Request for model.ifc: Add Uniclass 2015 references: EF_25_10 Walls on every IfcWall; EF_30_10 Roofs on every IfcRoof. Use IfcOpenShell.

First a look at what the model holds.

```python
import ifcopenshell

model = ifcopenshell.open("model.ifc")
print(model.schema)
print("classifications:", [c.Name for c in model.by_type("IfcClassification")])
for ifc_class in ("IfcDoor", "IfcRoof", "IfcStair", "IfcWall", "IfcWindow"):
    print(ifc_class, len(model.by_type(ifc_class)))
```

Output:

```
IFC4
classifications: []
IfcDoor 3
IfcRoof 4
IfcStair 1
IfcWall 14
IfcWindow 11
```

```python
import ifcopenshell
import ifcopenshell.api.classification

model = ifcopenshell.open("model.ifc")

system = ifcopenshell.api.classification.add_classification(model, classification="Uniclass 2015")

codes = {
    "IfcWall": ("EF_25_10", "Walls"),
    "IfcRoof": ("EF_30_10", "Roofs"),
}
for ifc_class, (code, name) in codes.items():
    products = model.by_type(ifc_class)
    ifcopenshell.api.classification.add_reference(
        model, products=products, classification=system, identification=code, name=name
    )
    print(code, len(products))

model.write("model_rev.ifc")
```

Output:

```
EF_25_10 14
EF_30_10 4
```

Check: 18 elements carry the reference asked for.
